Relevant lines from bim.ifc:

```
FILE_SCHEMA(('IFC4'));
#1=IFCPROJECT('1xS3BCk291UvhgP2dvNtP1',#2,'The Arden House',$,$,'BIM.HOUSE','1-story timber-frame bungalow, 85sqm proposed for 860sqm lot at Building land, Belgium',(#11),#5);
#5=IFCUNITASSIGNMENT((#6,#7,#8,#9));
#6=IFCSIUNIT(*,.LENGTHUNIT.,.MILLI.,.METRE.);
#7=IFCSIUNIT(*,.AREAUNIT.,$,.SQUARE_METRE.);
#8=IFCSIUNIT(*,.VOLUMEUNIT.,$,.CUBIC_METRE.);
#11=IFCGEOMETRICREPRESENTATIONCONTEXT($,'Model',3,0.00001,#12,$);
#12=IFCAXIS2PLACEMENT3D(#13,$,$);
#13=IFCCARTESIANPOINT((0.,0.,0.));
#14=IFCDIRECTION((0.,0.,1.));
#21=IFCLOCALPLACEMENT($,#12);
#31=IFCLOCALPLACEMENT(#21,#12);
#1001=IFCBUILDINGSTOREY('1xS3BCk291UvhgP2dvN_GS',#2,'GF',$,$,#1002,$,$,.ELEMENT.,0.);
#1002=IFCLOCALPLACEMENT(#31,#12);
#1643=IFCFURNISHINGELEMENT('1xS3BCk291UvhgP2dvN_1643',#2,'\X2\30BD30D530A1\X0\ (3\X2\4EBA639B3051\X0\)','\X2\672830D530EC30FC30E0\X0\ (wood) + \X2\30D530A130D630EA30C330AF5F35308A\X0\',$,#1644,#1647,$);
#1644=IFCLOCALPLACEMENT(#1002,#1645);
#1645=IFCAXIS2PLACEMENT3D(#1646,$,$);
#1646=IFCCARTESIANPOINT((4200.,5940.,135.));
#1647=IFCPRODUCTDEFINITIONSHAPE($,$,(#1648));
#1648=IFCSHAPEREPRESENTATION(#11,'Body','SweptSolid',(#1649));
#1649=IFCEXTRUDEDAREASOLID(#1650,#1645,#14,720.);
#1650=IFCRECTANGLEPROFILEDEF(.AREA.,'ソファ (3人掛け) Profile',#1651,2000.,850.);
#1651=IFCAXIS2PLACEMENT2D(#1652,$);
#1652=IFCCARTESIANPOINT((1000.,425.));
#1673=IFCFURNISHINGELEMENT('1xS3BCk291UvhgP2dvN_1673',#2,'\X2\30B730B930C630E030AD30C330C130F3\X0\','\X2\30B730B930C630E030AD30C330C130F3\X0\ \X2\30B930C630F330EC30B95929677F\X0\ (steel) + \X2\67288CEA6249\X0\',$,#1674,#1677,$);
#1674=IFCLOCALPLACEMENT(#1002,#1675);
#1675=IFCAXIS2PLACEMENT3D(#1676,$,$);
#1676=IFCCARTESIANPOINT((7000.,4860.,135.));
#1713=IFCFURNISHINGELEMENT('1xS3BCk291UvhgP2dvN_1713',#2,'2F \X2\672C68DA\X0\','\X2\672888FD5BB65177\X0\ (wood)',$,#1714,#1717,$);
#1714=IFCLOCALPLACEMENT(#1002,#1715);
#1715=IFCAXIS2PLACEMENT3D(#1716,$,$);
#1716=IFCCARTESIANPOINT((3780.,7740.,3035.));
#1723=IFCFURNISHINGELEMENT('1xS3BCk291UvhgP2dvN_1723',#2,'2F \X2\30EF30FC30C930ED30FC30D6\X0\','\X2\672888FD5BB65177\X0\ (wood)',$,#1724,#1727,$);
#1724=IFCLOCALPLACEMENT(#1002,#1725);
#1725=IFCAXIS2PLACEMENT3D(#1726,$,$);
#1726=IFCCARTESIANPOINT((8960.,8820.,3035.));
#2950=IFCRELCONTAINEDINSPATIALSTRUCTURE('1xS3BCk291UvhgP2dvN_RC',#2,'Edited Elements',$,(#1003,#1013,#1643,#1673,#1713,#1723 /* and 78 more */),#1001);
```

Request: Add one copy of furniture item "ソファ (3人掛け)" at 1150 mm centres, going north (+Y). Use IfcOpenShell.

```python
import numpy as np
import ifcopenshell
import ifcopenshell.api.geometry
import ifcopenshell.api.root
import ifcopenshell.util.element
import ifcopenshell.util.placement
import ifcopenshell.util.unit

model = ifcopenshell.open("bim.ifc")
unit_scale = ifcopenshell.util.unit.calculate_unit_scale(model)


def reuse_history(source, copy):
    """copy_class also copies each property set's owner history, people and application; keep the originals."""
    for rel in copy.IsDefinedBy:
        if rel.is_a("IfcRelDefinesByProperties") and (history := rel.RelatingPropertyDefinition.OwnerHistory):
            rel.RelatingPropertyDefinition.OwnerHistory = source.OwnerHistory
            ifcopenshell.util.element.remove_deep2(model, history)


source = model.by_id(1643)
base = ifcopenshell.util.placement.get_local_placement(source.ObjectPlacement)
step = np.array([0.0, 1.0, 0.0]) * 1.15 / unit_scale

for i in range(1, 2):
    copy = ifcopenshell.api.root.copy_class(model, product=source)
    copy.Representation = ifcopenshell.util.element.copy_deep(
        model, source.Representation, exclude=["IfcGeometricRepresentationContext", "IfcRepresentationMap"]
    )
    reuse_history(source, copy)
    matrix = base.copy()
    matrix[:3, 3] += i * step
    print("added at", matrix[:3, 3].round(3) + 0.0)
    ifcopenshell.api.geometry.edit_object_placement(model, product=copy, matrix=matrix, is_si=False)

model.write("bim_updated.ifc")
```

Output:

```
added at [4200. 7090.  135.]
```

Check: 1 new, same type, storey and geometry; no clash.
